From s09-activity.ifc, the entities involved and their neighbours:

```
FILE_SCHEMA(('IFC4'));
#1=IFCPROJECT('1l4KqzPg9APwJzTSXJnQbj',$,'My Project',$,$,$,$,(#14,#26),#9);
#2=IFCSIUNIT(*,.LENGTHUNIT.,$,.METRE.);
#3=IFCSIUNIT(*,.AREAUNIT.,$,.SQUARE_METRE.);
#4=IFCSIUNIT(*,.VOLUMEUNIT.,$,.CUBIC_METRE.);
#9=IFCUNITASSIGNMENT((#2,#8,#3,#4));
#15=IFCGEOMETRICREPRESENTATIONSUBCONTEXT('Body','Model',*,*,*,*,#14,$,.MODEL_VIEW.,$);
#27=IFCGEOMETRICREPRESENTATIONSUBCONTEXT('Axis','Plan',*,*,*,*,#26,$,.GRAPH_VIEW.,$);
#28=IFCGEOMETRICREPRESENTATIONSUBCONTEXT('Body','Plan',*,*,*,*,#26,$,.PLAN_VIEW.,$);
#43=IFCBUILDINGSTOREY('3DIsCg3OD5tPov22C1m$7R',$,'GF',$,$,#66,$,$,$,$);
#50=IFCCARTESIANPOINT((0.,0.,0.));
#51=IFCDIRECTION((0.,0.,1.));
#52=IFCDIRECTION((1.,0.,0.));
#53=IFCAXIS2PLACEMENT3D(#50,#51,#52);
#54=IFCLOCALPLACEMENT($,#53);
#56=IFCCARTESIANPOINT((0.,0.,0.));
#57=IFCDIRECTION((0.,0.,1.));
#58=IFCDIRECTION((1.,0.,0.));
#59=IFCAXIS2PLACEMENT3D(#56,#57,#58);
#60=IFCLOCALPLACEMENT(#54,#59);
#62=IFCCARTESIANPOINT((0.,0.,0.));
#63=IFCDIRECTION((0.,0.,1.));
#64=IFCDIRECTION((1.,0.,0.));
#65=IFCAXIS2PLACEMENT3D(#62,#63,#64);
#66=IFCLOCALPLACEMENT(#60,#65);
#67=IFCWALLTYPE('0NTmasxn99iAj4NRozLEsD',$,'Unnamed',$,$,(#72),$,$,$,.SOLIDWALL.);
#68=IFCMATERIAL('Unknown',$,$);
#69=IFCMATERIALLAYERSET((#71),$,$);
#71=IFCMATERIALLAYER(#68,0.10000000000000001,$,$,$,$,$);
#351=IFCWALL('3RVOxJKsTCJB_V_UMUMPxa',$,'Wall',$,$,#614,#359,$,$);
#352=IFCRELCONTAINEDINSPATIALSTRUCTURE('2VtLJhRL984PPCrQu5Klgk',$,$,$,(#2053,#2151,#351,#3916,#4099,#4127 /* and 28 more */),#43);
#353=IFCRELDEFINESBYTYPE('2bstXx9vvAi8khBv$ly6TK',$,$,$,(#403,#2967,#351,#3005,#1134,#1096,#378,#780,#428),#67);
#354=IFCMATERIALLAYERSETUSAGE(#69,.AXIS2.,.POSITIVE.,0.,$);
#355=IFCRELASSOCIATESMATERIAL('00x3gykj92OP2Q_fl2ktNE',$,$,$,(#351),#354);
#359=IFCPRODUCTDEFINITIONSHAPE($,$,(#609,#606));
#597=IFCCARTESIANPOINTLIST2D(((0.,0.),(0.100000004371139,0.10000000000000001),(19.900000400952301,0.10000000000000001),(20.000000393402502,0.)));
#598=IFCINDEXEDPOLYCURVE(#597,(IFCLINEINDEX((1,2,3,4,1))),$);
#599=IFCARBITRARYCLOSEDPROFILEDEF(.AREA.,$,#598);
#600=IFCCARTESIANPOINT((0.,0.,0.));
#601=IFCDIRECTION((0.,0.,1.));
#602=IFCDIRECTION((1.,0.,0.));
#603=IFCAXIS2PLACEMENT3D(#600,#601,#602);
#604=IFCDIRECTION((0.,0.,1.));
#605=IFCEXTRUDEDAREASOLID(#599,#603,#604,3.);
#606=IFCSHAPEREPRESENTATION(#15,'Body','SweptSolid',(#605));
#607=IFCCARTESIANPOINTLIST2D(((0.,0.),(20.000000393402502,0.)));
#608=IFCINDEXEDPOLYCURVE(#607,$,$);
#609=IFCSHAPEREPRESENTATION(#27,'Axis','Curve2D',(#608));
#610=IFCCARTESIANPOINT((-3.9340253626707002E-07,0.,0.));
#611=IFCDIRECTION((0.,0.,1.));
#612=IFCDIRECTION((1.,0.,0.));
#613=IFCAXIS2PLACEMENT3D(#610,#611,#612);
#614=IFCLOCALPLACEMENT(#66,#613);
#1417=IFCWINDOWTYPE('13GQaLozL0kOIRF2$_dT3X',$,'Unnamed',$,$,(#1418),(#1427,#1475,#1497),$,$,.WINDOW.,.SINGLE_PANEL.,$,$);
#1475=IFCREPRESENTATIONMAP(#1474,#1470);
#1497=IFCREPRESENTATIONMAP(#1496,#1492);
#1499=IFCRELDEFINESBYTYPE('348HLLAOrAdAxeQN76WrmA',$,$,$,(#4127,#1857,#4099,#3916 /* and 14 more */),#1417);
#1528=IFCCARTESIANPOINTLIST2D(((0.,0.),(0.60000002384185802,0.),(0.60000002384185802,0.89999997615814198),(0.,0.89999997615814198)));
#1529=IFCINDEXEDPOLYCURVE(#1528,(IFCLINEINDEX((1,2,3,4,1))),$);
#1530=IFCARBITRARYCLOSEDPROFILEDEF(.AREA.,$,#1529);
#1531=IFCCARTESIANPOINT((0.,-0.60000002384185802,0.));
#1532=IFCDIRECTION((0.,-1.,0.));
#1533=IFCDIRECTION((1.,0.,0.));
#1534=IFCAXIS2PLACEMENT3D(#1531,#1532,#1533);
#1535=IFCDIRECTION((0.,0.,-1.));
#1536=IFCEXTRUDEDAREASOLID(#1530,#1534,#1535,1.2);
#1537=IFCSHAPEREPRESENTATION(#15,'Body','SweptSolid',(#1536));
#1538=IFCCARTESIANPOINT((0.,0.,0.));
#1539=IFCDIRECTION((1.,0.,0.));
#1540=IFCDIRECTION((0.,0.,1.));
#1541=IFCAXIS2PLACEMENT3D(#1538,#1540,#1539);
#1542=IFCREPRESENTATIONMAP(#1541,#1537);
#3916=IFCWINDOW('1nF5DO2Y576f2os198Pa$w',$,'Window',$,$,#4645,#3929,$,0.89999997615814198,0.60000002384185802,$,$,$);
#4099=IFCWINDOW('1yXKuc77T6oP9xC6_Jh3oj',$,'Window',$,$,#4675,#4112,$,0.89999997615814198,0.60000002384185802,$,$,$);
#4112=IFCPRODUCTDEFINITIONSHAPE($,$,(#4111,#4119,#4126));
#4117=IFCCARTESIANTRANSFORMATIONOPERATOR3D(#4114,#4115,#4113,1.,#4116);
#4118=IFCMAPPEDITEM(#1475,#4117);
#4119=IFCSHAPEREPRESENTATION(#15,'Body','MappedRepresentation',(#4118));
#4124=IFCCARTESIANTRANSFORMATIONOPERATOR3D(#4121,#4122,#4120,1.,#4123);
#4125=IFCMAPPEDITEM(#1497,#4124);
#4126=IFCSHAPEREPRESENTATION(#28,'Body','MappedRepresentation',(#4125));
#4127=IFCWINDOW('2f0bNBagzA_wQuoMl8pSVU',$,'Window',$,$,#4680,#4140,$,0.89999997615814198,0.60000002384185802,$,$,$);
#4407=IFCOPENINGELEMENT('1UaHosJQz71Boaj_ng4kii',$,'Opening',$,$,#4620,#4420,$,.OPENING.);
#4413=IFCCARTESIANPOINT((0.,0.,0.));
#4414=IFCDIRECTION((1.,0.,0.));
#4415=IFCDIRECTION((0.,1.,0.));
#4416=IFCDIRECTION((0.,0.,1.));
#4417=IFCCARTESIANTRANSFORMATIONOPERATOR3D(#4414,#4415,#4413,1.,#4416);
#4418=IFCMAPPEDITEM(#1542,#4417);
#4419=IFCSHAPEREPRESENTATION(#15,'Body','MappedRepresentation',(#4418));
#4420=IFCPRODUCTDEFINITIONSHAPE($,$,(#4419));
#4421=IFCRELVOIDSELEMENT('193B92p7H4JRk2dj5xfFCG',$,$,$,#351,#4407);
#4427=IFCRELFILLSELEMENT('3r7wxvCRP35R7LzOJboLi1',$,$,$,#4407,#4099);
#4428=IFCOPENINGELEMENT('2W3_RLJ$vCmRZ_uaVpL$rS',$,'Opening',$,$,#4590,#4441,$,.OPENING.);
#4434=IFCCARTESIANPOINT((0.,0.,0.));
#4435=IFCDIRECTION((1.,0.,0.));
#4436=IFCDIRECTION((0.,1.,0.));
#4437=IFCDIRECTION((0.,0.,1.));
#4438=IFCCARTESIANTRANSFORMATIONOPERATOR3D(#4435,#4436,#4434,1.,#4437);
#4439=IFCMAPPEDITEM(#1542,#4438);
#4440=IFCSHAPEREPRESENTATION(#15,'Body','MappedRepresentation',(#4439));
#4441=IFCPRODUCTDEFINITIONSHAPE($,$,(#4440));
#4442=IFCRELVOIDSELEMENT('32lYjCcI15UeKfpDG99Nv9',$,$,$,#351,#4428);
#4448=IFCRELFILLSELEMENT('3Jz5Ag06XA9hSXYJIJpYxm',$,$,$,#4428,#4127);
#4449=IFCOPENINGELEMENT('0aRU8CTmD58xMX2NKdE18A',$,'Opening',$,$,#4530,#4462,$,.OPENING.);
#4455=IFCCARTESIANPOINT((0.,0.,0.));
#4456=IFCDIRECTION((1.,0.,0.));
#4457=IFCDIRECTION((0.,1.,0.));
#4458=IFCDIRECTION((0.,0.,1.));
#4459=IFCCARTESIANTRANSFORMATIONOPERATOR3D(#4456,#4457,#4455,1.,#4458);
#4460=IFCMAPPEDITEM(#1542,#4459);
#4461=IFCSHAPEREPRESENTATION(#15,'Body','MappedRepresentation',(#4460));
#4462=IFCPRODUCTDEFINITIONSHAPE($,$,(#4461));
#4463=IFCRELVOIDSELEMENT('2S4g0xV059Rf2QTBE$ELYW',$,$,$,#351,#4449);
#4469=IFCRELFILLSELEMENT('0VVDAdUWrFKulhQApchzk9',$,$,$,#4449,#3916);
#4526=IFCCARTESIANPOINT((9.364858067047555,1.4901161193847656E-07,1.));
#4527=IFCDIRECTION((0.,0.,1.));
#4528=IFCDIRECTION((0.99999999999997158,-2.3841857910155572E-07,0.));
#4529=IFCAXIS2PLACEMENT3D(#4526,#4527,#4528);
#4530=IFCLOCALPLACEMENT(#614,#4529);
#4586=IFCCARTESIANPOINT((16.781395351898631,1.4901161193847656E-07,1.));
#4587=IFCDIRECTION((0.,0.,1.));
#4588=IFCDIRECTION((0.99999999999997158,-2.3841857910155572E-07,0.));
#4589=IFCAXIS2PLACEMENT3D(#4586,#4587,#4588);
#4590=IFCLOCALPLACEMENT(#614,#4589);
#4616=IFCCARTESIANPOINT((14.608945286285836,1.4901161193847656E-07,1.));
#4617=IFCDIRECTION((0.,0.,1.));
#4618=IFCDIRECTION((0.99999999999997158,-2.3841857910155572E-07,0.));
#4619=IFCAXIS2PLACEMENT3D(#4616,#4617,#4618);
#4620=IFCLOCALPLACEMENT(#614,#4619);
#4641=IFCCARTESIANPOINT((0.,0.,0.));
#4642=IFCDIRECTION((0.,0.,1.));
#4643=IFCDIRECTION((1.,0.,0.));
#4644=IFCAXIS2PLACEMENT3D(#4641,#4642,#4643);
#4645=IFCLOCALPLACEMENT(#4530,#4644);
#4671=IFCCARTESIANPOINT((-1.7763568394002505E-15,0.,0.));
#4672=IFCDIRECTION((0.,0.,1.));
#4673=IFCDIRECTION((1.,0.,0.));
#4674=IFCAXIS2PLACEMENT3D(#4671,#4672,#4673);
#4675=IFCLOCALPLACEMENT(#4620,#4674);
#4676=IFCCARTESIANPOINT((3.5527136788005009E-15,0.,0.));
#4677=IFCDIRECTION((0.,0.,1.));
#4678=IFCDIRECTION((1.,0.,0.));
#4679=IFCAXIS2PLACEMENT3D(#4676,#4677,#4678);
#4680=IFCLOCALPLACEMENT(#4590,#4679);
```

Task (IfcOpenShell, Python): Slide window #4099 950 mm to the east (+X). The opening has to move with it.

```python
import ifcopenshell
import ifcopenshell.api.geometry
import ifcopenshell.util.placement
import ifcopenshell.util.unit

model = ifcopenshell.open("s09-activity.ifc")
unit_scale = ifcopenshell.util.unit.calculate_unit_scale(model)

window = model.by_guid("1yXKuc77T6oP9xC6_Jh3oj")
opening = window.FillsVoids[0].RelatingOpeningElement
wall = opening.VoidsElements[0].RelatingBuildingElement

wall_matrix = ifcopenshell.util.placement.get_local_placement(wall.ObjectPlacement)
shift = wall_matrix[:3, 0] * 0.95 / unit_scale
before = ifcopenshell.util.placement.get_local_placement(window.ObjectPlacement)[:3, 3].copy()

# The window is placed relative to its opening, so it follows when the opening moves.
matrix = ifcopenshell.util.placement.get_local_placement(opening.ObjectPlacement)
matrix[:3, 3] += shift
ifcopenshell.api.geometry.edit_object_placement(
    model, product=opening, matrix=matrix, is_si=False, should_transform_children=True
)

after = ifcopenshell.util.placement.get_local_placement(window.ObjectPlacement)[:3, 3]
print("window moved by", (after - before).round(3) + 0.0)

model.write("s09-activity_v2.ifc")
```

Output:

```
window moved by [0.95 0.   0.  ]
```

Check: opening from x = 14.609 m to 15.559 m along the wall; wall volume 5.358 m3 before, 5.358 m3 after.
